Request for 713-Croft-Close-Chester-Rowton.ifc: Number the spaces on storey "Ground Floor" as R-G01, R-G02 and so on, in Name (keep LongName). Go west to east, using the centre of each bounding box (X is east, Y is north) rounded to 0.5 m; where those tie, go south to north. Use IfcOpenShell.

First a look at what the model holds.

```python
import ifcopenshell
import ifcopenshell.util.element
import ifcopenshell.util.placement

model = ifcopenshell.open("713-Croft-Close-Chester-Rowton.ifc")
print(model.schema)
storey = next(s for s in model.by_type("IfcBuildingStorey") if s.Name == "Ground Floor")
spaces = [e for e in ifcopenshell.util.element.get_decomposition(storey) if e.is_a("IfcSpace")]
for e in sorted(spaces, key=lambda e: e.id()):
    origin = ifcopenshell.util.placement.get_local_placement(e.ObjectPlacement)[:3, 3]
    print(e.id(), e.Name, e.LongName, origin.round(2) + 0.0, sep=" | ")
```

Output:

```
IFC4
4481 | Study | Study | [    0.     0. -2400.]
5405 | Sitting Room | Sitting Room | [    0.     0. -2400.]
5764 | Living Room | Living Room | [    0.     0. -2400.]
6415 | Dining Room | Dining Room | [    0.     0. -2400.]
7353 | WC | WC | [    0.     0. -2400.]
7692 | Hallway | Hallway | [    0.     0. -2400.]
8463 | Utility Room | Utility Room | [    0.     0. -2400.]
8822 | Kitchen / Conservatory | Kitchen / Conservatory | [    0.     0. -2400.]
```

```python
import ifcopenshell
import ifcopenshell.geom
import ifcopenshell.util.element
import ifcopenshell.util.shape

model = ifcopenshell.open("713-Croft-Close-Chester-Rowton.ifc")
settings = ifcopenshell.geom.settings()
settings.set("use-world-coords", True)


def centre(element):
    shape = ifcopenshell.geom.create_shape(settings, element)
    return ifcopenshell.util.shape.get_bbox_centroid(shape.geometry)


storey = next(s for s in model.by_type("IfcBuildingStorey") if s.Name == "Ground Floor")
spaces = [e for e in ifcopenshell.util.element.get_decomposition(storey) if e.is_a("IfcSpace")]

# Insertion points can sit at a corner or the storey origin, so sort by the geometry (in metres).
centres = {e: centre(e) for e in spaces}
spaces.sort(key=lambda e: (round(centres[e][0] / 0.5), centres[e][1]))

for i, e in enumerate(spaces, start=1):
    number = f"R-G{i:02d}"
    e.Name = number
    print(e.id(), number)

model.write("713-Croft-Close-Chester-Rowton_edited.ifc")
```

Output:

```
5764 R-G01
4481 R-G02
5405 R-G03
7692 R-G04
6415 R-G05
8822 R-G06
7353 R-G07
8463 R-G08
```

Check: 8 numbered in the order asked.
